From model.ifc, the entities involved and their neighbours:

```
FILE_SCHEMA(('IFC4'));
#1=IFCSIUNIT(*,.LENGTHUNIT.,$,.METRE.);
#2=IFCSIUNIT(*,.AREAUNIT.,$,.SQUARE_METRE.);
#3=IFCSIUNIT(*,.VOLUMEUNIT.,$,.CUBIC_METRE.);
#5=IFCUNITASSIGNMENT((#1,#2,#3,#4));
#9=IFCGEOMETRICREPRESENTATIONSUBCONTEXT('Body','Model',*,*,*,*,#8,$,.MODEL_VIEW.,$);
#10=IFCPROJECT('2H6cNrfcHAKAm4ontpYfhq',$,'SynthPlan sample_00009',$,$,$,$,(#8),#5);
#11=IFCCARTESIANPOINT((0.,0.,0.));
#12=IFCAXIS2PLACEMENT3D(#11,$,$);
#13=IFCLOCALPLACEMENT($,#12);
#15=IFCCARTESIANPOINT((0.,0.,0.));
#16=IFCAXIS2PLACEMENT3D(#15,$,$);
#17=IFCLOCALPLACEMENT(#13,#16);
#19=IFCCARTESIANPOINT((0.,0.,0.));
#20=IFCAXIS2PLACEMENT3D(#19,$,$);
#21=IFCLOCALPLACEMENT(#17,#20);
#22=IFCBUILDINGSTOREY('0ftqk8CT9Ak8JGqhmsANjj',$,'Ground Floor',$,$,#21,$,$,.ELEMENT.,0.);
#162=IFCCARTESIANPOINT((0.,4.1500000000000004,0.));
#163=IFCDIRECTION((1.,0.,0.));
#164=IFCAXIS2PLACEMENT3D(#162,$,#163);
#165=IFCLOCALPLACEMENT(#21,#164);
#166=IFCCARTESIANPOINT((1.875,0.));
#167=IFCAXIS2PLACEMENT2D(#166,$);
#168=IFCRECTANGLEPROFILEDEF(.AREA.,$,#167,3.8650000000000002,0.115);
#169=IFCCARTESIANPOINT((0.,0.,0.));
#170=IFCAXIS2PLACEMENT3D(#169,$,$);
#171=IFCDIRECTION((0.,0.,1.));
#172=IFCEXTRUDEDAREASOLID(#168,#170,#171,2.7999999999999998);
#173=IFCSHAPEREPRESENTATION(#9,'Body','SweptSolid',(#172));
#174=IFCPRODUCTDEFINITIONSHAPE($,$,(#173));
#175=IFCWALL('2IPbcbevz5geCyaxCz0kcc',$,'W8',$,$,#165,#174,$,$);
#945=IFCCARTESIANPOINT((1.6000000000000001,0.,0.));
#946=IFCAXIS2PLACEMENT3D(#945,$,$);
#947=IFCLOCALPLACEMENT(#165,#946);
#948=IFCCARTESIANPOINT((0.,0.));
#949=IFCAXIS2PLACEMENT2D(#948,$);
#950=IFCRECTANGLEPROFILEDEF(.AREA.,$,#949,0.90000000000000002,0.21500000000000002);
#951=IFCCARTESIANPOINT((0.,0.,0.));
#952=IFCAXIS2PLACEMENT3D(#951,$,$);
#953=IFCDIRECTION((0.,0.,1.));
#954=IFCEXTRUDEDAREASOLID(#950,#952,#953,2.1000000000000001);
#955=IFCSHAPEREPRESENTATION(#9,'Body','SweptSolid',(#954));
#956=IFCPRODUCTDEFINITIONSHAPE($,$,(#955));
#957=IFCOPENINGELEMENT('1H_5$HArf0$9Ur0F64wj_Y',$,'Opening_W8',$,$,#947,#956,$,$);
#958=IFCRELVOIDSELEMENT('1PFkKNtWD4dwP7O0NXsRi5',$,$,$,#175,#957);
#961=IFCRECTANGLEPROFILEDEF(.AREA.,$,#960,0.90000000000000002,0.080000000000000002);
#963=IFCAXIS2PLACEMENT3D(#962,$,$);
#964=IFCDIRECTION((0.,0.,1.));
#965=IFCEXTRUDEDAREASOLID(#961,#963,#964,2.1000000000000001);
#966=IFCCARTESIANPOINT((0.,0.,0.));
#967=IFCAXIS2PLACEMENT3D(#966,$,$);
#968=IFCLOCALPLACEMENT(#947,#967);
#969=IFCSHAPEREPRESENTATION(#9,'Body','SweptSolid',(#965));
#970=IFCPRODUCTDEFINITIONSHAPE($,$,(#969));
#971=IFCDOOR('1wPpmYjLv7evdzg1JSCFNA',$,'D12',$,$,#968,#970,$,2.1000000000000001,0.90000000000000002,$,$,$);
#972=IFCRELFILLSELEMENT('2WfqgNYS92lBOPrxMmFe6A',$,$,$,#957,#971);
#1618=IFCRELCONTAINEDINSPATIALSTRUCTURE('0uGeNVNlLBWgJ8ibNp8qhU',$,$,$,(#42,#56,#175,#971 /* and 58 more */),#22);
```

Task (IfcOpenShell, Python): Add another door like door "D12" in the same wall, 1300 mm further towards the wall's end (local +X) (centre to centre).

```python
import ifcopenshell
import ifcopenshell.api.feature
import ifcopenshell.api.geometry
import ifcopenshell.api.root
import ifcopenshell.geom
import ifcopenshell.util.element
import ifcopenshell.util.placement
import ifcopenshell.util.shape
import ifcopenshell.util.unit

model = ifcopenshell.open("model.ifc")
unit_scale = ifcopenshell.util.unit.calculate_unit_scale(model)
settings = ifcopenshell.geom.settings()


def volume(element):
    """Net volume in cubic metres, openings subtracted."""
    shape = ifcopenshell.geom.create_shape(settings, element)
    return ifcopenshell.util.shape.get_volume(shape.geometry)


door = model.by_id(971)
opening = door.FillsVoids[0].RelatingOpeningElement
wall = opening.VoidsElements[0].RelatingBuildingElement
before = volume(wall)
shift = ifcopenshell.util.placement.get_local_placement(wall.ObjectPlacement)[:3, 0] * 1.3 / unit_scale

# copy_class copies the void relationship, type, container and properties, but no geometry.
new_opening = ifcopenshell.api.root.copy_class(model, product=opening)
new_opening.Representation = ifcopenshell.util.element.copy_deep(
    model, opening.Representation, exclude=["IfcGeometricRepresentationContext", "IfcRepresentationMap"]
)
new_door = ifcopenshell.api.root.copy_class(model, product=door)
new_door.Representation = ifcopenshell.util.element.copy_deep(
    model, door.Representation, exclude=["IfcGeometricRepresentationContext", "IfcRepresentationMap"]
)
ifcopenshell.api.feature.add_filling(model, opening=new_opening, element=new_door)

for old, new in ((opening, new_opening), (door, new_door)):
    matrix = ifcopenshell.util.placement.get_local_placement(old.ObjectPlacement)
    matrix[:3, 3] += shift
    ifcopenshell.api.geometry.edit_object_placement(model, product=new, matrix=matrix, is_si=False)

after = volume(wall)

print(f"wall volume {before:.3f} -> {after:.3f} m3")

model.write("model_rev.ifc")
```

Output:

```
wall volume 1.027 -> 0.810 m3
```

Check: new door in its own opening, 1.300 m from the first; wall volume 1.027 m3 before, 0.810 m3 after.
